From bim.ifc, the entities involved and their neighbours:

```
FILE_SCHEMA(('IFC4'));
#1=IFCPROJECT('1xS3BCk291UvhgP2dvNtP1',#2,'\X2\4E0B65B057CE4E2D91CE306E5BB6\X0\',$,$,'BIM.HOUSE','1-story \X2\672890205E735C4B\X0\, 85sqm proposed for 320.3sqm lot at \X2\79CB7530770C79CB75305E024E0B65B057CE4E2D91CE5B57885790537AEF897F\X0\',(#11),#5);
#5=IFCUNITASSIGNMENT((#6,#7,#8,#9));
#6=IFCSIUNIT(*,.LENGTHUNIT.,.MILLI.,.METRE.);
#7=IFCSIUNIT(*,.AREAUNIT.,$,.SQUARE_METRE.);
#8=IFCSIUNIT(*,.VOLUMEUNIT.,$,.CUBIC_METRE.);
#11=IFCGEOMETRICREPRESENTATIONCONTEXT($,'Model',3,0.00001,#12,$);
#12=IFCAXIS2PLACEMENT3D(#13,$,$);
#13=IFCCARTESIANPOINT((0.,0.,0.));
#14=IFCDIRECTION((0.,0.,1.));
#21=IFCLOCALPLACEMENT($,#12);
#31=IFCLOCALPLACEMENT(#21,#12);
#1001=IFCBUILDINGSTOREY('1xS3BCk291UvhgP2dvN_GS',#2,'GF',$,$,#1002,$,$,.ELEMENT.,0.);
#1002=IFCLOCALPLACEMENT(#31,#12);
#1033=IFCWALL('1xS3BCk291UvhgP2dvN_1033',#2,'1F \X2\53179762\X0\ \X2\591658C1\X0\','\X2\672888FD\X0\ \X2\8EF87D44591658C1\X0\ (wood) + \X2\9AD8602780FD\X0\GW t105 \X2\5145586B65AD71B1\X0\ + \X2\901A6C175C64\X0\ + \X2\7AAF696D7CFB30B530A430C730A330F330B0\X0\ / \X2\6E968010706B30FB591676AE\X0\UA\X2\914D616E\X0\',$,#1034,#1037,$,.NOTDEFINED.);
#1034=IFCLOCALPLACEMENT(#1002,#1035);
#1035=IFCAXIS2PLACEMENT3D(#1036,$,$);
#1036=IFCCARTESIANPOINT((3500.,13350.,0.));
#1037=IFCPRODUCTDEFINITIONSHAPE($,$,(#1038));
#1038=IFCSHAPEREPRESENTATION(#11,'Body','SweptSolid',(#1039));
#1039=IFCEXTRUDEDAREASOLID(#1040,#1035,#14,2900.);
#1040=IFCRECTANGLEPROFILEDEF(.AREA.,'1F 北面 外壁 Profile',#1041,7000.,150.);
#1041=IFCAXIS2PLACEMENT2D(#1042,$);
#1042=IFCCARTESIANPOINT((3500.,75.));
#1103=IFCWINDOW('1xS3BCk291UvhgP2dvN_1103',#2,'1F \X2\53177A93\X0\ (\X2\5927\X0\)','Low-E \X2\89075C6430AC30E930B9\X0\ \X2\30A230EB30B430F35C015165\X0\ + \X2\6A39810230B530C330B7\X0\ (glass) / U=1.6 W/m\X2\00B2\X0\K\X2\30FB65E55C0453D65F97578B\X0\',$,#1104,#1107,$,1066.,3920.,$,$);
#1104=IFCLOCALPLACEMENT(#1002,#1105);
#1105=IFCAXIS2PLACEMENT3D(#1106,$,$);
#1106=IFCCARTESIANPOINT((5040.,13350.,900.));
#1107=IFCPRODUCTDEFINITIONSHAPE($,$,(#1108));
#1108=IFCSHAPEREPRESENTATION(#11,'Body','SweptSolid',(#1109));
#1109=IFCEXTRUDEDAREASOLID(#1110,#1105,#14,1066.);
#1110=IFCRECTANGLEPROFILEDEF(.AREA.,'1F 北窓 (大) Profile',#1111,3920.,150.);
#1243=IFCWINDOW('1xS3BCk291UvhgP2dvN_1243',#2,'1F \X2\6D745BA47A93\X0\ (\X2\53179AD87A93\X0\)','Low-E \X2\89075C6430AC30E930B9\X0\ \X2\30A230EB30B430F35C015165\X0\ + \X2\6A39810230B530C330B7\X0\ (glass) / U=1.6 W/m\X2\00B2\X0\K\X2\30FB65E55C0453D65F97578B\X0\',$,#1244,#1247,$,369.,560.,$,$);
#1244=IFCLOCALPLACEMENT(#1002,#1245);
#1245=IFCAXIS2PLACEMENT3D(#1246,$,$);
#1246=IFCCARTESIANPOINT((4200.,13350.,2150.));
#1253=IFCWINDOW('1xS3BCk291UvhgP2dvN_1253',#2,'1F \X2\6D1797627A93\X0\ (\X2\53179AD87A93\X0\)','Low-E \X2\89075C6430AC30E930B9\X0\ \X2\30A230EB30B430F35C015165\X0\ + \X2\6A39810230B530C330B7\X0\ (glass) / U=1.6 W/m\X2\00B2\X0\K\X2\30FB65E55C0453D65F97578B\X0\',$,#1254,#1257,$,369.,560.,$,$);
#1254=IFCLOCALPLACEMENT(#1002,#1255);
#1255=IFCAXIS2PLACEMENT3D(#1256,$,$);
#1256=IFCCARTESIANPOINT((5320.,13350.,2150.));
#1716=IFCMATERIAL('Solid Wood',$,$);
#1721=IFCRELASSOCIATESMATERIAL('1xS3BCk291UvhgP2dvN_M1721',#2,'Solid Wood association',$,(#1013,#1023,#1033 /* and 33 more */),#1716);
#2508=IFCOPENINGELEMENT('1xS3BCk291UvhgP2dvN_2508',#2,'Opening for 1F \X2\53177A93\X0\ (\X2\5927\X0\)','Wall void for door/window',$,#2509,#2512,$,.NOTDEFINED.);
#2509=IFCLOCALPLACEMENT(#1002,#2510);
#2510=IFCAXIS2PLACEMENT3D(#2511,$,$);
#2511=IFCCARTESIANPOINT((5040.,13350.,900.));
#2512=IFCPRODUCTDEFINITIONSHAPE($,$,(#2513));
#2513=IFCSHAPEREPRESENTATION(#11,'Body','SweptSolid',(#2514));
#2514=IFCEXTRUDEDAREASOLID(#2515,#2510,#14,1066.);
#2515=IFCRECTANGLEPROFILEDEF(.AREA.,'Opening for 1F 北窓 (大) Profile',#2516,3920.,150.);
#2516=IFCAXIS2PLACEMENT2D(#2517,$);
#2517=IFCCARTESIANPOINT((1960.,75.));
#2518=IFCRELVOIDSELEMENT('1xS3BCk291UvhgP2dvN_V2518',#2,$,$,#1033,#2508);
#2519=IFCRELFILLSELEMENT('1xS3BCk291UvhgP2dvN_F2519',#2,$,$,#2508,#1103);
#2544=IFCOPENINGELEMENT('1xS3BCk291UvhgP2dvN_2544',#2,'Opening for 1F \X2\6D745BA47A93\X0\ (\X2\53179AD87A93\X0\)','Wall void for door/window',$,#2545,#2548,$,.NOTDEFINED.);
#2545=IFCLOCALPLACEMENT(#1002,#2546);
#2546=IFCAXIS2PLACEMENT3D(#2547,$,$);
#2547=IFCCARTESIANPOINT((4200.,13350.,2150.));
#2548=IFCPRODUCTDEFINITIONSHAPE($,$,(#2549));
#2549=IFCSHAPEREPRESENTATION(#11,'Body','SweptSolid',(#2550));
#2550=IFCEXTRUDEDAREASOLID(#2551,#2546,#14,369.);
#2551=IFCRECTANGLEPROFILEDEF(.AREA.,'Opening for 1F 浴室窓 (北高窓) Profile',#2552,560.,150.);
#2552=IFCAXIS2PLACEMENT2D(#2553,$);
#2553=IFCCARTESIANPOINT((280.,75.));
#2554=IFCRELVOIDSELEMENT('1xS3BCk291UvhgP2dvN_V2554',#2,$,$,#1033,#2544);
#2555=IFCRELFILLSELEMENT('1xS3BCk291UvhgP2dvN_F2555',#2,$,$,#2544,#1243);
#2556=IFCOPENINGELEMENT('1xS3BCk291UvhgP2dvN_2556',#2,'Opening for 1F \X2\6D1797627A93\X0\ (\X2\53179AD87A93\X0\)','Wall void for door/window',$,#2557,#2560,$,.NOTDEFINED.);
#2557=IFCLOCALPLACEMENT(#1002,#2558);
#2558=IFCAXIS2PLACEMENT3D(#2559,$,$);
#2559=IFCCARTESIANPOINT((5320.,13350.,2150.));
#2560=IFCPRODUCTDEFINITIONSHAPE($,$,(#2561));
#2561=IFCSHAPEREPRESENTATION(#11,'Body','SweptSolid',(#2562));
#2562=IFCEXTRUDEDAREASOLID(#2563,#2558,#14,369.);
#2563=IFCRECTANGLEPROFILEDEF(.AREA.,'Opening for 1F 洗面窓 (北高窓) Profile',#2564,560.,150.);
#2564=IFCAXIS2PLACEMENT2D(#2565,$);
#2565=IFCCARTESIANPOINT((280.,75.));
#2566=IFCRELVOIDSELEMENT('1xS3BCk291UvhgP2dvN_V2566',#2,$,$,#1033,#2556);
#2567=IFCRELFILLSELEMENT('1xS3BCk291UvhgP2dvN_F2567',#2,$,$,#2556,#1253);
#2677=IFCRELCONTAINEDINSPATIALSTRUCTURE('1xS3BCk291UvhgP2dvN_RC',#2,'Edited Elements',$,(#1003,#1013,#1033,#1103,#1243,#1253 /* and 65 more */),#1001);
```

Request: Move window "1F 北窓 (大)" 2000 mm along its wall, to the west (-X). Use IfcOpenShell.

```python
import ifcopenshell
import ifcopenshell.api.geometry
import ifcopenshell.util.placement
import ifcopenshell.util.unit

model = ifcopenshell.open("bim.ifc")
unit_scale = ifcopenshell.util.unit.calculate_unit_scale(model)

window = model.by_guid("1xS3BCk291UvhgP2dvN_1103")
opening = window.FillsVoids[0].RelatingOpeningElement
wall = opening.VoidsElements[0].RelatingBuildingElement

wall_matrix = ifcopenshell.util.placement.get_local_placement(wall.ObjectPlacement)
shift = wall_matrix[:3, 0] * -2 / unit_scale
before = ifcopenshell.util.placement.get_local_placement(window.ObjectPlacement)[:3, 3].copy()

# The window is not placed relative to its opening, so move both.
for product in (opening, window):
    matrix = ifcopenshell.util.placement.get_local_placement(product.ObjectPlacement)
    matrix[:3, 3] += shift
    ifcopenshell.api.geometry.edit_object_placement(model, product=product, matrix=matrix, is_si=False)

after = ifcopenshell.util.placement.get_local_placement(window.ObjectPlacement)[:3, 3]
print("window moved by", (after - before).round(3) + 0.0)

model.write("bim_v2.ifc")
```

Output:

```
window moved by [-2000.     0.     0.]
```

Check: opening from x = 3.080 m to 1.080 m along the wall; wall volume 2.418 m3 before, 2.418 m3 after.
